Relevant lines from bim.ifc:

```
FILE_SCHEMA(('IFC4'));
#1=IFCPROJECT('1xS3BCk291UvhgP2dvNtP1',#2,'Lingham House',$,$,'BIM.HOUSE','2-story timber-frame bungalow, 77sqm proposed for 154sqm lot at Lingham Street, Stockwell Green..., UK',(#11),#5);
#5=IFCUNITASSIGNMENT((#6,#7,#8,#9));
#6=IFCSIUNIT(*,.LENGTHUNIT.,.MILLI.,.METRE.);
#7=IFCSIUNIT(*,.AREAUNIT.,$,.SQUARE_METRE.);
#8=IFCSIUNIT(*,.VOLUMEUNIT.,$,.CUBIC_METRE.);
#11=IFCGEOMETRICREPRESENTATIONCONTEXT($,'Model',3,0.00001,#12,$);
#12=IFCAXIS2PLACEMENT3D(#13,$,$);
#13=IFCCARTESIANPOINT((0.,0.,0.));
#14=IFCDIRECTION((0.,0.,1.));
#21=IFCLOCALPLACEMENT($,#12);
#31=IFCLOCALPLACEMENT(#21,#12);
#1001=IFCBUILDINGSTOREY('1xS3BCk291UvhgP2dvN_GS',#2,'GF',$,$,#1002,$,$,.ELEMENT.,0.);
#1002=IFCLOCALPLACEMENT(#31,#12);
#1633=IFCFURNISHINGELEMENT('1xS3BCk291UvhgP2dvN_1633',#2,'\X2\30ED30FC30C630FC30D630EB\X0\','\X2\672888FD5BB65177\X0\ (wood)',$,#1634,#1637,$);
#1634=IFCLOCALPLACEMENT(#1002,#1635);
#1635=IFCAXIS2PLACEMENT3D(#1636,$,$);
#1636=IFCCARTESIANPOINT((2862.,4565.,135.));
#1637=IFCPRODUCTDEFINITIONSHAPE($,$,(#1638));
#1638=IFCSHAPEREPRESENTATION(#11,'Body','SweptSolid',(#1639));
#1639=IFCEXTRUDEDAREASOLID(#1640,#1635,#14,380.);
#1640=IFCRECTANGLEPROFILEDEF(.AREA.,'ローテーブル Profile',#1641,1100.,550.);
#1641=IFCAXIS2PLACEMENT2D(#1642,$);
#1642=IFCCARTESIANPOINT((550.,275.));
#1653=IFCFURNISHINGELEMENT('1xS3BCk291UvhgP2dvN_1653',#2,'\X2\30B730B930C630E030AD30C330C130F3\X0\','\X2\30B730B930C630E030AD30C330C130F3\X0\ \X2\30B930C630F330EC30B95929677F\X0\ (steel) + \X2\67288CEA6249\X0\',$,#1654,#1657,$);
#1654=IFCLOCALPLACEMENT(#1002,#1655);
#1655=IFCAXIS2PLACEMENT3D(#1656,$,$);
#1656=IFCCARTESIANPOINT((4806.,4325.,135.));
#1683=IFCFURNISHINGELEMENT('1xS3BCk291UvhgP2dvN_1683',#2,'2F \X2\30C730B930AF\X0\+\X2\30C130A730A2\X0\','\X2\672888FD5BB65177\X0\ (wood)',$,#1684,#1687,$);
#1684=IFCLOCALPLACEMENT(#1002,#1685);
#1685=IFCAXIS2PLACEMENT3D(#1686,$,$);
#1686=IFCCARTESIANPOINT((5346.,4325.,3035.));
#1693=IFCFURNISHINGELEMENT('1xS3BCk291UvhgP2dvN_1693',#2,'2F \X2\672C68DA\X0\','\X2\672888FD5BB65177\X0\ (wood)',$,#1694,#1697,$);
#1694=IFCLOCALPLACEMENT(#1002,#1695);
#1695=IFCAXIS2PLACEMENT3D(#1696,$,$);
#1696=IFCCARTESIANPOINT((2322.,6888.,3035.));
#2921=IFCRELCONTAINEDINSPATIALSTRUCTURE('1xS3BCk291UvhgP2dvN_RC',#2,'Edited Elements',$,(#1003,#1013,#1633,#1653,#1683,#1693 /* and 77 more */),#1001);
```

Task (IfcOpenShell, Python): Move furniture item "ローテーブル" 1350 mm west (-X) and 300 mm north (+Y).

```python
import ifcopenshell
import ifcopenshell.api.geometry
import ifcopenshell.util.placement
import ifcopenshell.util.unit

model = ifcopenshell.open("bim.ifc")
unit_scale = ifcopenshell.util.unit.calculate_unit_scale(model)

item = model.by_id(1633)
matrix = ifcopenshell.util.placement.get_local_placement(item.ObjectPlacement)
matrix[0, 3] -= 1.35 / unit_scale
matrix[1, 3] += 0.3 / unit_scale
ifcopenshell.api.geometry.edit_object_placement(model, product=item, matrix=matrix, is_si=False)

print(ifcopenshell.util.placement.get_local_placement(item.ObjectPlacement).round(3) + 0.0)

model.write("bim_updated.ifc")
```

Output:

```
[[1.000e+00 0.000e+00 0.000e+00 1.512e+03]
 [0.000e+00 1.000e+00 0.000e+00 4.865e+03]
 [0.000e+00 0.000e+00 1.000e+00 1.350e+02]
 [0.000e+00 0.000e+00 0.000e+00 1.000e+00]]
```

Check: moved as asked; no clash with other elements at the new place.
